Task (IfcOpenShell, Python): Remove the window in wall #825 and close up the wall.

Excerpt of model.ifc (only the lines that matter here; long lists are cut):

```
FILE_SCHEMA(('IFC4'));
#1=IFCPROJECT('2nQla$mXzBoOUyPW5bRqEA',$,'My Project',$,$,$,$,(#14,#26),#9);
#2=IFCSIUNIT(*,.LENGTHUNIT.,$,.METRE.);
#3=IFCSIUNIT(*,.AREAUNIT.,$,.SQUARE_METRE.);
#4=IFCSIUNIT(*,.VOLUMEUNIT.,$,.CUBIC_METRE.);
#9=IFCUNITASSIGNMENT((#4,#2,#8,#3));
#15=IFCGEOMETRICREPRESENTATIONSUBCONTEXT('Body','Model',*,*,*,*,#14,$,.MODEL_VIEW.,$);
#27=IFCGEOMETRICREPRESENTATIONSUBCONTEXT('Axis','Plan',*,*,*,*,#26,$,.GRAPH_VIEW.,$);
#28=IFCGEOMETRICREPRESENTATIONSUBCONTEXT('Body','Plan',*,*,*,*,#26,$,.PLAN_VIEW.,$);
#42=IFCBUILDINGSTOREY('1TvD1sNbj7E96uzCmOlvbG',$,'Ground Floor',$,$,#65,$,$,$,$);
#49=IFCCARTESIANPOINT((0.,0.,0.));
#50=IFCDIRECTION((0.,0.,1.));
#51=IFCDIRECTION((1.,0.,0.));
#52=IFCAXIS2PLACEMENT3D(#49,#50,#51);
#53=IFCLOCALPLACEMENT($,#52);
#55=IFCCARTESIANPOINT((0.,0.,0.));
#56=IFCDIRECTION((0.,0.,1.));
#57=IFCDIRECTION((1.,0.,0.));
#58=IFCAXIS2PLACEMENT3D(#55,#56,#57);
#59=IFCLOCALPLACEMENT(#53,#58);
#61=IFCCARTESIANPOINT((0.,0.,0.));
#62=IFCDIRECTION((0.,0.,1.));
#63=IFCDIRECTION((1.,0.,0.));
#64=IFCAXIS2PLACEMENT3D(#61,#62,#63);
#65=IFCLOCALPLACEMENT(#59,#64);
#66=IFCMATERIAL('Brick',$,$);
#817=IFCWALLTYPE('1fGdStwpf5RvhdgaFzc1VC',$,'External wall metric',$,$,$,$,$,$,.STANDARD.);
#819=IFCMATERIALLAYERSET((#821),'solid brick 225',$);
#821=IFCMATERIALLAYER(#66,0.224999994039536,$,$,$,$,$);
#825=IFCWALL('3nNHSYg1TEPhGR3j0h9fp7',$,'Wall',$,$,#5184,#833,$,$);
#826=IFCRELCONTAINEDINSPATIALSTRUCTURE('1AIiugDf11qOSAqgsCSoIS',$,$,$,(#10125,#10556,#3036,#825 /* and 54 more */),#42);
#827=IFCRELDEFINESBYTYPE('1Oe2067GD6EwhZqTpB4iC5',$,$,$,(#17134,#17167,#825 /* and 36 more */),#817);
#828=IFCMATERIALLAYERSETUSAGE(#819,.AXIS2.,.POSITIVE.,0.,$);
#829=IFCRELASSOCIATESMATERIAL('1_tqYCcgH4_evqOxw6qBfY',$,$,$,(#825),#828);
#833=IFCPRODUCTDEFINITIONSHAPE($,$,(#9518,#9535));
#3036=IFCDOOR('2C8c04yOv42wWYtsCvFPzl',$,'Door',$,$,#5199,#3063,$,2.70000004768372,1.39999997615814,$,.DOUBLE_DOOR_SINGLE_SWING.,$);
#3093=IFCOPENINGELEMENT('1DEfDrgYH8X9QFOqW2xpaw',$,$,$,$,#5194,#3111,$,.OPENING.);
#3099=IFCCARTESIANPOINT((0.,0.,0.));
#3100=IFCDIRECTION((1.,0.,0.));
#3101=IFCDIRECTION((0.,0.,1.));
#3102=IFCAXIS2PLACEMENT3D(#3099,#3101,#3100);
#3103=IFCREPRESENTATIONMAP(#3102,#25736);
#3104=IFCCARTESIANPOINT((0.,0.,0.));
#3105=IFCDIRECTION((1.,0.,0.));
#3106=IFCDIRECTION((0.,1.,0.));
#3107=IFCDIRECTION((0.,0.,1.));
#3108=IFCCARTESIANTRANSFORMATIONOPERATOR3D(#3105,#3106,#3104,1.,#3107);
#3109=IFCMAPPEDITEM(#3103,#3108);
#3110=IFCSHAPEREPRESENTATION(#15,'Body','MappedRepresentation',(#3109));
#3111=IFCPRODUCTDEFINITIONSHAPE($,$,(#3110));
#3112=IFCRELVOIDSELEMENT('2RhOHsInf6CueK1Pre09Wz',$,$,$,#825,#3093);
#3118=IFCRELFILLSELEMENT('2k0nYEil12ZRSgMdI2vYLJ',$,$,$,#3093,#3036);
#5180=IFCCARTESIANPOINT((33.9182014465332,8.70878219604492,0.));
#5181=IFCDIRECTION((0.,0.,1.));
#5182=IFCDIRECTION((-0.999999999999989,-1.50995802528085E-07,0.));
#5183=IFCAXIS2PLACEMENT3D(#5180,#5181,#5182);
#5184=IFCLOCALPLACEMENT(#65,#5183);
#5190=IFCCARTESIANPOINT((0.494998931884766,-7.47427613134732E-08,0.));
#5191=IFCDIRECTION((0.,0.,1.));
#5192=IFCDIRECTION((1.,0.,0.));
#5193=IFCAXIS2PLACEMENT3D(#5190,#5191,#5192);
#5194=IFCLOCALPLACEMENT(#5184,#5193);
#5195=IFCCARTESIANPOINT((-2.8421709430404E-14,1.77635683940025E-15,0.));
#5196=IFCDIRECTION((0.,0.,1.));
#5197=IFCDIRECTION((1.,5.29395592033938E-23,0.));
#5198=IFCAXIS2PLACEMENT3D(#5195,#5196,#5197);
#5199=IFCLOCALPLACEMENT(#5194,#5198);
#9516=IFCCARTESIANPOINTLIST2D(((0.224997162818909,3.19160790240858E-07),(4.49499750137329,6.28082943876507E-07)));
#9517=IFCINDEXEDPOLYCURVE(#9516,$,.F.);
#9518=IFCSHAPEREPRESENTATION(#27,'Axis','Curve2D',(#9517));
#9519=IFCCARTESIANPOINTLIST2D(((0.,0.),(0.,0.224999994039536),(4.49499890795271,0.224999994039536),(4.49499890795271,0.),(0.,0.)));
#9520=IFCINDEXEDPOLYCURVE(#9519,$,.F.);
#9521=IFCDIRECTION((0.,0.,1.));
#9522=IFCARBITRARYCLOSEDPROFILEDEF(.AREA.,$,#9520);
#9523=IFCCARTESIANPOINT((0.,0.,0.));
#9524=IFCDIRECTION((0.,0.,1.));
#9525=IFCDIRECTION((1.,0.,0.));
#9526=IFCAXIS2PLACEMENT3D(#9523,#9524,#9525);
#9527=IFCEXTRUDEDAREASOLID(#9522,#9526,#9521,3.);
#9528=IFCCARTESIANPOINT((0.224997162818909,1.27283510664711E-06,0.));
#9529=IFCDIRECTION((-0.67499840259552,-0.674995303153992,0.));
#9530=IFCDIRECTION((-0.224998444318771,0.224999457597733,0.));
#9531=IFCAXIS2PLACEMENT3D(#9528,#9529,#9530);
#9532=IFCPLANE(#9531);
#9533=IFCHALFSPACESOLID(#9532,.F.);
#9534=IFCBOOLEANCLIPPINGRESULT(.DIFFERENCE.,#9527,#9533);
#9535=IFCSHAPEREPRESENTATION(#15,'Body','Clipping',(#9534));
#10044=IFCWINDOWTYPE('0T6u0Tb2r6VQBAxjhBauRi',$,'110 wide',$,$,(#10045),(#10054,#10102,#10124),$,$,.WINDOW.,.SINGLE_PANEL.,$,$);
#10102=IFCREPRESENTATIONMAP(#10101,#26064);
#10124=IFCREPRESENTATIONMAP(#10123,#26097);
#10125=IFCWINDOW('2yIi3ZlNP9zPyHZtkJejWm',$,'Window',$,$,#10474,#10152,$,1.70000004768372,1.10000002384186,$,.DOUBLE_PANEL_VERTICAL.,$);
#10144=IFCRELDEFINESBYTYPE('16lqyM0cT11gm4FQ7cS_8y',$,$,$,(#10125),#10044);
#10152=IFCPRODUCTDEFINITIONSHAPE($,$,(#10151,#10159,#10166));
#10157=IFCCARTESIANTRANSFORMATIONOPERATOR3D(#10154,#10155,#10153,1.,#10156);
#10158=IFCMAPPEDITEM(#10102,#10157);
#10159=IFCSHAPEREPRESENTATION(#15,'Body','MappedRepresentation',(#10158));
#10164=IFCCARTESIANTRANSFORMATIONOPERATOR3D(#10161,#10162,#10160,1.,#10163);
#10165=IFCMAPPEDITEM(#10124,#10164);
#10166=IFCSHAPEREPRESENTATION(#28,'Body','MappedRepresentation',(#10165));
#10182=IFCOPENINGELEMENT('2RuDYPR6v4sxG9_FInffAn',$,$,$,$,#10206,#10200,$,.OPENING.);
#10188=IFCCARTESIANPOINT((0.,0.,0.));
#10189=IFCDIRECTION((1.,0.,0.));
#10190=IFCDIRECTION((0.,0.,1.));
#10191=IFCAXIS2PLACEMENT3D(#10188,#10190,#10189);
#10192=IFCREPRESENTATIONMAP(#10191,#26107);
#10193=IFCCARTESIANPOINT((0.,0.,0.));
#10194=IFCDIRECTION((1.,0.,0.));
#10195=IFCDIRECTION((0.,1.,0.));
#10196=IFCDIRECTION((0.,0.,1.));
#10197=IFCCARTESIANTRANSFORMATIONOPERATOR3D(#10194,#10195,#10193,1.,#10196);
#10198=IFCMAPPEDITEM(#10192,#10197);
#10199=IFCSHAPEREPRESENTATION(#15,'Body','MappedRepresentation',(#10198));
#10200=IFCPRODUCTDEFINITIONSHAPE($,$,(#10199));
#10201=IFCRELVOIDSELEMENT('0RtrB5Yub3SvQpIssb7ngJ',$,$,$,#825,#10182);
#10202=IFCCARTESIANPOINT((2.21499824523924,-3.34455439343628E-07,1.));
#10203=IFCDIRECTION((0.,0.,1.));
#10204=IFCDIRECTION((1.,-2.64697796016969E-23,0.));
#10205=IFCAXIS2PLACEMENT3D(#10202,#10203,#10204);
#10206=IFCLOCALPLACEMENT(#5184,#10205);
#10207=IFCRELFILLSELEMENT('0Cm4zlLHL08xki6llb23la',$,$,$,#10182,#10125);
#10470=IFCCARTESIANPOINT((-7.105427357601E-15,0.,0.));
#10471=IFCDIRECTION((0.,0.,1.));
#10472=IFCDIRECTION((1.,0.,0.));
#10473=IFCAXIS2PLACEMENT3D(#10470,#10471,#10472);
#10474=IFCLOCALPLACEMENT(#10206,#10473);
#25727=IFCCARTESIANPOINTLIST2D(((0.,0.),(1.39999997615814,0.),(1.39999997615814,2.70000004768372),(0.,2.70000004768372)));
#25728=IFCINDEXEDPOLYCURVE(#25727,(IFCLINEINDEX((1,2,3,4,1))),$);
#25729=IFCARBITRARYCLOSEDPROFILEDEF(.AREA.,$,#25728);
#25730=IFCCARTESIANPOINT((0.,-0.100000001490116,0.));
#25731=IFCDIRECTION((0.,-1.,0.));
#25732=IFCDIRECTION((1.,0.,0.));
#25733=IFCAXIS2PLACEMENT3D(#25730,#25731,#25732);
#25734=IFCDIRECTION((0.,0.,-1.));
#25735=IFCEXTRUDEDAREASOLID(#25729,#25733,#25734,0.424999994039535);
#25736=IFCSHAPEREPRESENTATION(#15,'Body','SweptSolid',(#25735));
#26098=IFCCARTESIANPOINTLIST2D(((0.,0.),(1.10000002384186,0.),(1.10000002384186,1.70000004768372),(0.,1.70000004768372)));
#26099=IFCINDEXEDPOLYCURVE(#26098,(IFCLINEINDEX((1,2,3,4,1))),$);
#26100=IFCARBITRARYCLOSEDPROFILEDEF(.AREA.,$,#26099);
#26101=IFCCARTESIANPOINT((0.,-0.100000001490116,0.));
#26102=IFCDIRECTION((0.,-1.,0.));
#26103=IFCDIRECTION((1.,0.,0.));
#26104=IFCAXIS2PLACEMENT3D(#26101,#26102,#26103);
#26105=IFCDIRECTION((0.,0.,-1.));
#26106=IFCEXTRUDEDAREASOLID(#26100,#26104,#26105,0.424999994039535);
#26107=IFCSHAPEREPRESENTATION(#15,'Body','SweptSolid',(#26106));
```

```python
import ifcopenshell
import ifcopenshell.api.feature
import ifcopenshell.api.root
import ifcopenshell.geom
import ifcopenshell.util.shape

model = ifcopenshell.open("model.ifc")
settings = ifcopenshell.geom.settings()


def volume(element):
    """Net volume in cubic metres, openings subtracted."""
    shape = ifcopenshell.geom.create_shape(settings, element)
    return ifcopenshell.util.shape.get_volume(shape.geometry)


window = model.by_guid("2yIi3ZlNP9zPyHZtkJejWm")
opening = window.FillsVoids[0].RelatingOpeningElement
wall = opening.VoidsElements[0].RelatingBuildingElement
before = volume(wall)

ifcopenshell.api.root.remove_product(model, product=window)
ifcopenshell.api.feature.remove_feature(model, feature=opening)

after = volume(wall)

print(f"wall volume {before:.3f} -> {after:.3f} m3")

model.write("model_updated.ifc")
```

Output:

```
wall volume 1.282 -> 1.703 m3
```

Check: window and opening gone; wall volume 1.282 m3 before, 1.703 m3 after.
